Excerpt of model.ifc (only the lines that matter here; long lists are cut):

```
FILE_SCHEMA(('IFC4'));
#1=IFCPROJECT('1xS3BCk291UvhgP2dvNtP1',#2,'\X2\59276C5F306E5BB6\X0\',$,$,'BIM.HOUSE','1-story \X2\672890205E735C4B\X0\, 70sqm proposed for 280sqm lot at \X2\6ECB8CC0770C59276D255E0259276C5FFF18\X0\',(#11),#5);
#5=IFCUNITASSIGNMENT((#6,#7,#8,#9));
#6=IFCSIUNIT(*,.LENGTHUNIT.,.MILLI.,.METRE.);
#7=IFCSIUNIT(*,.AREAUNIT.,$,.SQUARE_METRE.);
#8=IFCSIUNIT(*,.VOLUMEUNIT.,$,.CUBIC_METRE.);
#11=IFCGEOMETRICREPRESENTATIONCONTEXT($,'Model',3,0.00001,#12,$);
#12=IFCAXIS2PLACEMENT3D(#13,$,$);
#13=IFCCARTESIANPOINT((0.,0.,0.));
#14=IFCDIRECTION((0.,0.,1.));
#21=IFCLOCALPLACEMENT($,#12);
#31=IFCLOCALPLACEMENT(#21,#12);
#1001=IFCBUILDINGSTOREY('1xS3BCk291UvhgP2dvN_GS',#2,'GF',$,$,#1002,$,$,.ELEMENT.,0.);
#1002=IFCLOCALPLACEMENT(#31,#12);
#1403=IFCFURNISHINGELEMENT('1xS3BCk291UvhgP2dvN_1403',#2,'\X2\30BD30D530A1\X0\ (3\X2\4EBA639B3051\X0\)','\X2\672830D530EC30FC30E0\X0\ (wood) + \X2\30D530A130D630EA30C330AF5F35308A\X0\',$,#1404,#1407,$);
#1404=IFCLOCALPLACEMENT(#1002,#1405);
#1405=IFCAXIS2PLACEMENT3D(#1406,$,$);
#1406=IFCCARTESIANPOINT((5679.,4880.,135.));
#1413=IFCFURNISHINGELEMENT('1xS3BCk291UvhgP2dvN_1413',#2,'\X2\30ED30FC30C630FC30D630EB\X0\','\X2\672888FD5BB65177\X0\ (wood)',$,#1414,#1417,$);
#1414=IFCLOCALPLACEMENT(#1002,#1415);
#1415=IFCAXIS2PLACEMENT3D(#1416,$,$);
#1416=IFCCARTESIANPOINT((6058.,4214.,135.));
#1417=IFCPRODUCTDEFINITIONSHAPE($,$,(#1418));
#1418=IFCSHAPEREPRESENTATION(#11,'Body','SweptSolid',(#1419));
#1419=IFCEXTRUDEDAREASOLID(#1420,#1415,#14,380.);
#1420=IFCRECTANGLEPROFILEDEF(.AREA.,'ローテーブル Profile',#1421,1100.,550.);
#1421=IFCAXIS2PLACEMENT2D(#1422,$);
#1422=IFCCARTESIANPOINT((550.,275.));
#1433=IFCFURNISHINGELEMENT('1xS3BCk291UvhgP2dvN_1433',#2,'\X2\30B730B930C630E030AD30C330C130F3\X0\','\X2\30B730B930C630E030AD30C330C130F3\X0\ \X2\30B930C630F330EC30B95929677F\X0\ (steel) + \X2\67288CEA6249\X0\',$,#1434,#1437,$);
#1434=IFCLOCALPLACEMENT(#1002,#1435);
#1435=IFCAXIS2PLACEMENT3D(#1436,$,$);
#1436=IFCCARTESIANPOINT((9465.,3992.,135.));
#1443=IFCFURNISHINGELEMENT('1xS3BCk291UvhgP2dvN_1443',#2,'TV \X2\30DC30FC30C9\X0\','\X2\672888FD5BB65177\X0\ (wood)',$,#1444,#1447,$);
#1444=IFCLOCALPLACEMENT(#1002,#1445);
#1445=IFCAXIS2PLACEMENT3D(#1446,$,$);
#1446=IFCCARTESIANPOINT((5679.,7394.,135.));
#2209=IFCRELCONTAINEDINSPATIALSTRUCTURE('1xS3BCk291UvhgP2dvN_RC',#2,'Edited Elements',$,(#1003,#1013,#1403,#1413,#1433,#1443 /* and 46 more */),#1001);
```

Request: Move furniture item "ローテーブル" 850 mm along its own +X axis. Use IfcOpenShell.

```python
import ifcopenshell
import ifcopenshell.api.geometry
import ifcopenshell.util.placement
import ifcopenshell.util.unit

model = ifcopenshell.open("model.ifc")
unit_scale = ifcopenshell.util.unit.calculate_unit_scale(model)

item = model.by_id(1413)
matrix = ifcopenshell.util.placement.get_local_placement(item.ObjectPlacement)
matrix[:3, 3] += matrix[:3, 0] * 0.85 / unit_scale
ifcopenshell.api.geometry.edit_object_placement(model, product=item, matrix=matrix, is_si=False)

print(ifcopenshell.util.placement.get_local_placement(item.ObjectPlacement).round(3) + 0.0)

model.write("model_v2.ifc")
```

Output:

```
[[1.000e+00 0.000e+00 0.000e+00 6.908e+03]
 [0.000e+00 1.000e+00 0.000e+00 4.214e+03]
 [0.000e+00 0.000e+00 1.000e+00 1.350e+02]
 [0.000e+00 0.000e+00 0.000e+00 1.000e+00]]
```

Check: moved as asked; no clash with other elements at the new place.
